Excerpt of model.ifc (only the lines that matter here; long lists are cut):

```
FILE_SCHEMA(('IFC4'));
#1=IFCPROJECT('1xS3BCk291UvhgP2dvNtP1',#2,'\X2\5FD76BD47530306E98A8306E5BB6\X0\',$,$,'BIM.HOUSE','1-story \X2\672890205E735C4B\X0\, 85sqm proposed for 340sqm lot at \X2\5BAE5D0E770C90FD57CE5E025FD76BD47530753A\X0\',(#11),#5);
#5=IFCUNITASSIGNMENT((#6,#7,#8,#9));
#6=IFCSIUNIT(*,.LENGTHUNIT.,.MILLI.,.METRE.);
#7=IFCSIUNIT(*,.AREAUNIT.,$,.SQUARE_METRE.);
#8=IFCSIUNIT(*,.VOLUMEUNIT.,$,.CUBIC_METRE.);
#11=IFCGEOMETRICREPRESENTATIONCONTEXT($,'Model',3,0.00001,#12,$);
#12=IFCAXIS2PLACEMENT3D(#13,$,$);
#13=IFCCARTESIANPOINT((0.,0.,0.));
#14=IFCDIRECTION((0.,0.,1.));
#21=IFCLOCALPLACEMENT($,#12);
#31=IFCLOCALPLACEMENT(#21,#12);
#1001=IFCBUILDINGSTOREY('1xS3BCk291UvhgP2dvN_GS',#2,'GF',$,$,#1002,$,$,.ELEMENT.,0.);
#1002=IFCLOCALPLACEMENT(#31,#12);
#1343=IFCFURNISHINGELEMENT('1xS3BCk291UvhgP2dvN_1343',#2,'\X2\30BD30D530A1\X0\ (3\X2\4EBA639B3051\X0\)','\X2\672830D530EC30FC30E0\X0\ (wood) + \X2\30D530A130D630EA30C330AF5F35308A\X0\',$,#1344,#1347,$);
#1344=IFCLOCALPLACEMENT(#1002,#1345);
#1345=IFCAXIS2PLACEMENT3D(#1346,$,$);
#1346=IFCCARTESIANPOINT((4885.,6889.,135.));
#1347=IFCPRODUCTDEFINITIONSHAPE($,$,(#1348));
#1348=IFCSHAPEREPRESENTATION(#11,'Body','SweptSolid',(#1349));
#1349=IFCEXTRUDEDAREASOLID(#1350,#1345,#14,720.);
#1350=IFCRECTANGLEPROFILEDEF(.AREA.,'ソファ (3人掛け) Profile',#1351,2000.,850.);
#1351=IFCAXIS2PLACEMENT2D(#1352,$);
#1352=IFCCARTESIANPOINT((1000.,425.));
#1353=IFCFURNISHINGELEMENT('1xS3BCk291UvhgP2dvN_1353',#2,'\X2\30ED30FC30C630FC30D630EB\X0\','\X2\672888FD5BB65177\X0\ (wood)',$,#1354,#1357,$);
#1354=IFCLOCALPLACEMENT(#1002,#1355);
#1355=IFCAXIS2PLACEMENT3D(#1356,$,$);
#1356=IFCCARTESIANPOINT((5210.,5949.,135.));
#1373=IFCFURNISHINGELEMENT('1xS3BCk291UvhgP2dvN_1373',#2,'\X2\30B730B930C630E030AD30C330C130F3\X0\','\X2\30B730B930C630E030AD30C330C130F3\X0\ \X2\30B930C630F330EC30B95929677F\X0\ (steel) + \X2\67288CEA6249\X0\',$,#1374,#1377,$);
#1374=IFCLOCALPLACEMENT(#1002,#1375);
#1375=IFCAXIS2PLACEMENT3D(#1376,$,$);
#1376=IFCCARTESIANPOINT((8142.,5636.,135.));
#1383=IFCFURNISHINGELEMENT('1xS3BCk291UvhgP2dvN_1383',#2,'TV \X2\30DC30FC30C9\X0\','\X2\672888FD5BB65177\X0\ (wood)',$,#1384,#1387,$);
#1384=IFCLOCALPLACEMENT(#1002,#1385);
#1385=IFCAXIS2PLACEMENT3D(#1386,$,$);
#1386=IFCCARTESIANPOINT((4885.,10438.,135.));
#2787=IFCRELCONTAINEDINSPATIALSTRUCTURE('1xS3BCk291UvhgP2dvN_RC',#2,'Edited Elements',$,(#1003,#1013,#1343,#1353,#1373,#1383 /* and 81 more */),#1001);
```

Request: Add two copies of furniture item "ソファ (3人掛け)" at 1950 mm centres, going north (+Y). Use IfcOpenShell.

```python
import numpy as np
import ifcopenshell
import ifcopenshell.api.geometry
import ifcopenshell.api.root
import ifcopenshell.util.element
import ifcopenshell.util.placement

model = ifcopenshell.open("model.ifc")


def reuse_history(source, copy):
    """copy_class also copies each property set's owner history, people and application; keep the originals."""
    for rel in copy.IsDefinedBy:
        if rel.is_a("IfcRelDefinesByProperties") and (history := rel.RelatingPropertyDefinition.OwnerHistory):
            rel.RelatingPropertyDefinition.OwnerHistory = source.OwnerHistory
            ifcopenshell.util.element.remove_deep2(model, history)


source = model.by_guid("1xS3BCk291UvhgP2dvN_1343")
base = ifcopenshell.util.placement.get_local_placement(source.ObjectPlacement)
step = np.array([0.0, 1.0, 0.0]) * 1950.0

for i in range(1, 3):
    copy = ifcopenshell.api.root.copy_class(model, product=source)
    copy.Representation = ifcopenshell.util.element.copy_deep(
        model, source.Representation, exclude=["IfcGeometricRepresentationContext", "IfcRepresentationMap"]
    )
    reuse_history(source, copy)
    matrix = base.copy()
    matrix[:3, 3] += i * step
    print("added at", matrix[:3, 3].round(3) + 0.0)
    ifcopenshell.api.geometry.edit_object_placement(model, product=copy, matrix=matrix, is_si=False)

model.write("model_v2.ifc")
```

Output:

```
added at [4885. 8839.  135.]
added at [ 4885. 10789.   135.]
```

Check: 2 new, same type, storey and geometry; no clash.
